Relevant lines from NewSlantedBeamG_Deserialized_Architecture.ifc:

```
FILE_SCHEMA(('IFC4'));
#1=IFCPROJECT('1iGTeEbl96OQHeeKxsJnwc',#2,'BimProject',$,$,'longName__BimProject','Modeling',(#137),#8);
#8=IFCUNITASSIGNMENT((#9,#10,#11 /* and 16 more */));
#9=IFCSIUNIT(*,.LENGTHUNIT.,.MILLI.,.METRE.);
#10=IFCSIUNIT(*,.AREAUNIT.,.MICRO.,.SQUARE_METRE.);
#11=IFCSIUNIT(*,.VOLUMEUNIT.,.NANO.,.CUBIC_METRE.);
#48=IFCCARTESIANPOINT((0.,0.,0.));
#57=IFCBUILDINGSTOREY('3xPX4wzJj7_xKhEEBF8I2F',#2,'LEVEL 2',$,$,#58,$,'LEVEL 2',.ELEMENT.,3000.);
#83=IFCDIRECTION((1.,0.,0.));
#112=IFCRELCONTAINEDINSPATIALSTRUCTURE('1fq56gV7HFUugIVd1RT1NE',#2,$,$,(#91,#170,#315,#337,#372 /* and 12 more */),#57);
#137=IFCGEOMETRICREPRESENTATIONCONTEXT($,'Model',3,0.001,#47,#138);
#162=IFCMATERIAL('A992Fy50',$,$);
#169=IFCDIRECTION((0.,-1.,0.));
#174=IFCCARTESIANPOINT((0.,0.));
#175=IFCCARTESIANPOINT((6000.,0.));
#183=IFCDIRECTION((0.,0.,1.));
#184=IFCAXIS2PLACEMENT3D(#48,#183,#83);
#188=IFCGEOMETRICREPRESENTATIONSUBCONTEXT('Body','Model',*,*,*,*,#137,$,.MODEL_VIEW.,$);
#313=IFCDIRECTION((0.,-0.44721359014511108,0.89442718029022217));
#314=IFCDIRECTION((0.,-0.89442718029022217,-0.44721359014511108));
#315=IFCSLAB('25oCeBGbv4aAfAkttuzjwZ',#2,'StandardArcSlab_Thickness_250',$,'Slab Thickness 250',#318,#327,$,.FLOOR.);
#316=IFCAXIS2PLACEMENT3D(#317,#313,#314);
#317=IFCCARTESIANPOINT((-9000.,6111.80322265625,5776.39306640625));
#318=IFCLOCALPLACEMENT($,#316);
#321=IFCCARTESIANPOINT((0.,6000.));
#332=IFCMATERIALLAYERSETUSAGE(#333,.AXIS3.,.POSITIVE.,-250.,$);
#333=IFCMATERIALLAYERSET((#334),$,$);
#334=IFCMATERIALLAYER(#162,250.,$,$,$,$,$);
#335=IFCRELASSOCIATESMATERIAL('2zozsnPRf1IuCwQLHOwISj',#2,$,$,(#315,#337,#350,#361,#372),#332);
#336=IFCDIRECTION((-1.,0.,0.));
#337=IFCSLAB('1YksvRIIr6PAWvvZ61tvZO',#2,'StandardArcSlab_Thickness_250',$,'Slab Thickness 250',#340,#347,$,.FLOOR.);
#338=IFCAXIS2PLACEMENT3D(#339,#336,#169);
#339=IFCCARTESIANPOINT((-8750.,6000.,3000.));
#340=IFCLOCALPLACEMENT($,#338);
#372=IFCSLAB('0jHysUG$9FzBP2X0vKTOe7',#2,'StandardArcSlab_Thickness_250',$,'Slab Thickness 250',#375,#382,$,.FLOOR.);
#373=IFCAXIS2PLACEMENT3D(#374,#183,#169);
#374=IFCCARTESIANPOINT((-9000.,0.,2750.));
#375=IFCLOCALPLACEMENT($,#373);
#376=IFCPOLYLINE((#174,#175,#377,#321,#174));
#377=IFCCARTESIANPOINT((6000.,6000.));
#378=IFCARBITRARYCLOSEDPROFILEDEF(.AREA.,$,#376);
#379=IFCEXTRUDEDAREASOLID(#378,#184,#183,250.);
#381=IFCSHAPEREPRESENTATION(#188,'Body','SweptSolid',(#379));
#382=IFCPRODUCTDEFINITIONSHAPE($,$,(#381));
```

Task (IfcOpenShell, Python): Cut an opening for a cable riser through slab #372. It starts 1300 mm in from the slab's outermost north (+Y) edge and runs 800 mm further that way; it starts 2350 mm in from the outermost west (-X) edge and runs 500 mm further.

```python
import numpy as np
import ifcopenshell
import ifcopenshell.api.feature
import ifcopenshell.api.geometry
import ifcopenshell.api.root
import ifcopenshell.geom
import ifcopenshell.util.placement
import ifcopenshell.util.representation
import ifcopenshell.util.shape
import ifcopenshell.util.unit

model = ifcopenshell.open("NewSlantedBeamG_Deserialized_Architecture.ifc")
unit_scale = ifcopenshell.util.unit.calculate_unit_scale(model)
settings = ifcopenshell.geom.settings()


def volume(element):
    """Net volume in cubic metres, openings subtracted."""
    shape = ifcopenshell.geom.create_shape(settings, element)
    return ifcopenshell.util.shape.get_volume(shape.geometry)


slab = model.by_guid("0jHysUG$9FzBP2X0vKTOe7")
before = volume(slab)

# Extent in the slab's own axes, in metres. The edges named are its -X and -Y sides.
slab_shape = ifcopenshell.geom.create_shape(settings, slab)
vertices = ifcopenshell.util.shape.get_vertices(slab_shape.geometry)
x_min, y_min, bottom = vertices.min(axis=0)
top = vertices[:, 2].max()

opening = ifcopenshell.api.root.create_entity(model, ifc_class="IfcOpeningElement", name="Cable riser opening", predefined_type="OPENING")
context = ifcopenshell.util.representation.get_context(model, "Model", "Body", "MODEL_VIEW")
width, depth = 0.8, 0.5
outline = [(0.0, 0.0), (width, 0.0), (width, depth), (0.0, depth), (0.0, 0.0)]
# Overshoot both faces by 50 mm so the cut is clean.
shape = ifcopenshell.api.geometry.add_slab_representation(
    model, context=context, depth=top - bottom + 0.1, polyline=outline
)
ifcopenshell.api.geometry.assign_representation(model, product=opening, representation=shape)

matrix = ifcopenshell.util.placement.get_local_placement(slab.ObjectPlacement)
matrix[:, 3] = matrix @ np.append(np.array([x_min + 1.3, y_min + 2.35, bottom - 0.05]) / unit_scale, 1.0)
ifcopenshell.api.geometry.edit_object_placement(model, product=opening, matrix=matrix, is_si=False)
ifcopenshell.api.feature.add_feature(model, feature=opening, element=slab)

after = volume(slab)

print(f"slab volume {before:.3f} -> {after:.3f} m3")

model.write("NewSlantedBeamG_Deserialized_Architecture_updated.ifc")
```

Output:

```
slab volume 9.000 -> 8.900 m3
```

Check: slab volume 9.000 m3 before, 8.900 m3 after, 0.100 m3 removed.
